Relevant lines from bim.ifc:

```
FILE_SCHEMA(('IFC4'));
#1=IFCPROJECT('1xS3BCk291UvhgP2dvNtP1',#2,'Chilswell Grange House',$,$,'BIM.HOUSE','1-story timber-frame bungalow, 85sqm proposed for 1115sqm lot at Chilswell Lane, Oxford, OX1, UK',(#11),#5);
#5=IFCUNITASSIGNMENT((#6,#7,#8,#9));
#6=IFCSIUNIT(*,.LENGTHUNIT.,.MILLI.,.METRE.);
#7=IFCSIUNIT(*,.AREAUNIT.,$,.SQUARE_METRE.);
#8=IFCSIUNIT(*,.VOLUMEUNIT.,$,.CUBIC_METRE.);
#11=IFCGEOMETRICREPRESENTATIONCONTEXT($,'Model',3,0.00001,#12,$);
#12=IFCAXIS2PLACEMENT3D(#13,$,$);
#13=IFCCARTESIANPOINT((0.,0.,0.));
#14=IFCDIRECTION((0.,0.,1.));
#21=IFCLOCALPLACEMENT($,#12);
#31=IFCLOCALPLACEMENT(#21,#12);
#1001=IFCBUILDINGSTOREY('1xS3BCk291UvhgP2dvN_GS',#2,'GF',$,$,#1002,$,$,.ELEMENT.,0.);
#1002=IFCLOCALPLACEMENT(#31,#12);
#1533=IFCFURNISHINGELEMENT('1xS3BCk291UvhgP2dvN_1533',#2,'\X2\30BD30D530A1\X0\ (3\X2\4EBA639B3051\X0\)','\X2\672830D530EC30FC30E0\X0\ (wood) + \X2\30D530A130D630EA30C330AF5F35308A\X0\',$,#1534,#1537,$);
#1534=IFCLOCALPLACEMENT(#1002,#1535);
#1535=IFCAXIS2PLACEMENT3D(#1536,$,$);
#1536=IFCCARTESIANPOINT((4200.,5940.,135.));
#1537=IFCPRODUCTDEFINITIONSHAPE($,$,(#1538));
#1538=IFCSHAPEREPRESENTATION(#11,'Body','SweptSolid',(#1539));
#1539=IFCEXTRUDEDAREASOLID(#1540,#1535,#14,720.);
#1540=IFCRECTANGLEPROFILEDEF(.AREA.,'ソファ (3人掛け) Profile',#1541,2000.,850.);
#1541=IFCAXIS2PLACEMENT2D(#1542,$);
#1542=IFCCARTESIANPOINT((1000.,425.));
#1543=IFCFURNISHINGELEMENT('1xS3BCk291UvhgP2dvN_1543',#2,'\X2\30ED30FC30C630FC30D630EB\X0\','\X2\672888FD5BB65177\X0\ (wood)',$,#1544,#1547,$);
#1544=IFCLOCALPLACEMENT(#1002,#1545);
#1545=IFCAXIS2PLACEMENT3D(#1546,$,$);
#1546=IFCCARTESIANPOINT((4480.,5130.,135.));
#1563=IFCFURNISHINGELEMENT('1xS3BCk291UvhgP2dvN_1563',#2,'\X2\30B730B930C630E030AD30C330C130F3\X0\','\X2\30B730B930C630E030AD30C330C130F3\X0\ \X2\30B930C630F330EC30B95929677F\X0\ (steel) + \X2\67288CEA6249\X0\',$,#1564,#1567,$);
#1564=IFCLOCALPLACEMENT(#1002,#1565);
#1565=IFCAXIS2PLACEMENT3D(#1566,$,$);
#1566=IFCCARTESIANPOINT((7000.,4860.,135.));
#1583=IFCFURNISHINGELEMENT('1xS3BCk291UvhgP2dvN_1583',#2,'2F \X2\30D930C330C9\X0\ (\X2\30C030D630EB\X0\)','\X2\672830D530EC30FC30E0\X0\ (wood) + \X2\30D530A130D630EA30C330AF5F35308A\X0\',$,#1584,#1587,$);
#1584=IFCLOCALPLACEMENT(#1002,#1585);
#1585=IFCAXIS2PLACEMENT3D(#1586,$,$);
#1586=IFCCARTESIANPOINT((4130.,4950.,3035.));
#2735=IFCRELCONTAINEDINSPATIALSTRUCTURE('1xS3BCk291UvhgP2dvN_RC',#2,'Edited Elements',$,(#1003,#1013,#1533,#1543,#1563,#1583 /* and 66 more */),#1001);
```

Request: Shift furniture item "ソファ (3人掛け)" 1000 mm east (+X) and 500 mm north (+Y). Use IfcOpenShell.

```python
import ifcopenshell
import ifcopenshell.api.geometry
import ifcopenshell.util.placement

model = ifcopenshell.open("bim.ifc")

item = model.by_guid("1xS3BCk291UvhgP2dvN_1533")
matrix = ifcopenshell.util.placement.get_local_placement(item.ObjectPlacement)
matrix[0, 3] += 1000.0
matrix[1, 3] += 500.0
ifcopenshell.api.geometry.edit_object_placement(model, product=item, matrix=matrix, is_si=False)

print(ifcopenshell.util.placement.get_local_placement(item.ObjectPlacement).round(3) + 0.0)

model.write("bim-out.ifc")
```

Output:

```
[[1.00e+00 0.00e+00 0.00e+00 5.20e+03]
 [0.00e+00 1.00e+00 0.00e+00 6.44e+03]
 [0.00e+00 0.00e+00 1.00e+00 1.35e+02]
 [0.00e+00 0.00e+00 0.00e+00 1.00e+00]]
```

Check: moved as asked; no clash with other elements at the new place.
